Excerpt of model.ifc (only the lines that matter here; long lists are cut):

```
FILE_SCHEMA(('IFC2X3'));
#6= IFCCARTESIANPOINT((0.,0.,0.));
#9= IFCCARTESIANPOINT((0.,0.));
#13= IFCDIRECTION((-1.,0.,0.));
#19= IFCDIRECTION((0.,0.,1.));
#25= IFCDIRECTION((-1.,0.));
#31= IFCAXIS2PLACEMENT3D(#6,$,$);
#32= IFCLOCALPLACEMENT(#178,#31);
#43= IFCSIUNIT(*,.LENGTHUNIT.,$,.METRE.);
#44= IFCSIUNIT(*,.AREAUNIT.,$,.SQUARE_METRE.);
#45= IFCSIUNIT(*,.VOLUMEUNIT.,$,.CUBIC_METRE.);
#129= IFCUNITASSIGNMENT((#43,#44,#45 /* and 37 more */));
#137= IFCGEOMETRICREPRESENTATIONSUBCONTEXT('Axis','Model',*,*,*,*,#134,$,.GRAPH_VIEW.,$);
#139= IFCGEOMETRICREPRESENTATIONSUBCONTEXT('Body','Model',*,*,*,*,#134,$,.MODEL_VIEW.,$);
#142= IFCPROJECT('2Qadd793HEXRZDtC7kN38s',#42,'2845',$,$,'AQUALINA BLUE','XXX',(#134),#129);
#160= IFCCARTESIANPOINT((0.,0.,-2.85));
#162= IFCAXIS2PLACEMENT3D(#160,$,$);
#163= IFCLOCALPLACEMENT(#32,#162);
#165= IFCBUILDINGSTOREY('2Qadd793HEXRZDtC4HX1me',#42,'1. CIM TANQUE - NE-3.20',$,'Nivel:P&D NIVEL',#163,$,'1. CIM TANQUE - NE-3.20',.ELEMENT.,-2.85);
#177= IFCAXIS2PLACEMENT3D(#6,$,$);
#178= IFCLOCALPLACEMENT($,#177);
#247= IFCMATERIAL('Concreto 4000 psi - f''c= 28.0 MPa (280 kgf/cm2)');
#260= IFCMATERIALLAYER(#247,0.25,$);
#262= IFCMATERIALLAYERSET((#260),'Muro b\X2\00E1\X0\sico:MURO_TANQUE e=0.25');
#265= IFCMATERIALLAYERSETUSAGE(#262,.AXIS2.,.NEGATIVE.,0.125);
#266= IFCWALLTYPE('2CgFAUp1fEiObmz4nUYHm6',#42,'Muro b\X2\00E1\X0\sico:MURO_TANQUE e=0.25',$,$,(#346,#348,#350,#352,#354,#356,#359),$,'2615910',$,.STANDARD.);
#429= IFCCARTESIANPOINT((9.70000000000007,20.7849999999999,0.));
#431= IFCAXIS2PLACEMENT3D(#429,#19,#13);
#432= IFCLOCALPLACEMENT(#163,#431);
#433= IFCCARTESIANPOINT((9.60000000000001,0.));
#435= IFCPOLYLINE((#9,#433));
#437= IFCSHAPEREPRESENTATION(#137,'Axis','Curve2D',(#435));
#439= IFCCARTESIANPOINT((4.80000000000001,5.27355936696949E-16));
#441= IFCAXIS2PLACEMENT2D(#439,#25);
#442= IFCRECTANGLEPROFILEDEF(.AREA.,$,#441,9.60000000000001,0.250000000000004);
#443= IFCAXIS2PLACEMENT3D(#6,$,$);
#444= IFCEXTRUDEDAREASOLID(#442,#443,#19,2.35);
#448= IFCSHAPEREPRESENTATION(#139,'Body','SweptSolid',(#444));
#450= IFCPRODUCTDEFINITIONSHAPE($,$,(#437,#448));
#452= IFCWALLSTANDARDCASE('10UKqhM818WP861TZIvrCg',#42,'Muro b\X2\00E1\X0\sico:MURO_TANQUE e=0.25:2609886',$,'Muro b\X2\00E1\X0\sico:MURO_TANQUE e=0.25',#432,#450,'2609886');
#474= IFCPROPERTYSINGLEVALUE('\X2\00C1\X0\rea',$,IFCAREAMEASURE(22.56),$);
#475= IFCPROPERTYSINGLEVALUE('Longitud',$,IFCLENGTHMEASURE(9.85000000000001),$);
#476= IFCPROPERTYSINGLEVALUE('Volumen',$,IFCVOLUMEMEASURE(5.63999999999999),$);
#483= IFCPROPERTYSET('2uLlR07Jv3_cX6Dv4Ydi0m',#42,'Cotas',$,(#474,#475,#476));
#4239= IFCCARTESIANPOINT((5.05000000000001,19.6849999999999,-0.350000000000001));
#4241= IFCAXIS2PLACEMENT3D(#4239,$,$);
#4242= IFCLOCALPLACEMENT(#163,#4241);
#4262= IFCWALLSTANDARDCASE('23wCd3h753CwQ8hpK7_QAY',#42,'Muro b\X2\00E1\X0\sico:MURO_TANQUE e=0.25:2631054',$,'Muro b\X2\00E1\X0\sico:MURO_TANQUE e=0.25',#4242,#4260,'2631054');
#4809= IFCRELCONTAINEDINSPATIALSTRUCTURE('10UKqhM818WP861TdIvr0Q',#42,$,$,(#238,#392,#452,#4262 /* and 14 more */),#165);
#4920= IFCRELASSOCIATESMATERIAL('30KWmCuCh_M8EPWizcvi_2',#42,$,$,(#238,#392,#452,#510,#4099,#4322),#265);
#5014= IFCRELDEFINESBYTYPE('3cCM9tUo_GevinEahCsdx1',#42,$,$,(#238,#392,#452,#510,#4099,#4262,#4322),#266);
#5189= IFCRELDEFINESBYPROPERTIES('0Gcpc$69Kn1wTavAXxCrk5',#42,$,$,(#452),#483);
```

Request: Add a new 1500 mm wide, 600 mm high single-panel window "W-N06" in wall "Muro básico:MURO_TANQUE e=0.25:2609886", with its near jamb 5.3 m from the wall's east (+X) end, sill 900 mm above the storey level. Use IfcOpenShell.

```python
import numpy as np
import ifcopenshell
import ifcopenshell.api.feature
import ifcopenshell.api.geometry
import ifcopenshell.api.pset
import ifcopenshell.api.root
import ifcopenshell.api.spatial
import ifcopenshell.api.type
import ifcopenshell.geom
import ifcopenshell.util.element
import ifcopenshell.util.placement
import ifcopenshell.util.representation
import ifcopenshell.util.shape
import ifcopenshell.util.unit

model = ifcopenshell.open("model.ifc")
unit_scale = ifcopenshell.util.unit.calculate_unit_scale(model)
area_scale = ifcopenshell.util.unit.calculate_unit_scale(model, "AREAUNIT")
volume_scale = ifcopenshell.util.unit.calculate_unit_scale(model, "VOLUMEUNIT")
settings = ifcopenshell.geom.settings()


def volume(element):
    """Net volume in cubic metres, openings subtracted."""
    shape = ifcopenshell.geom.create_shape(settings, element)
    return ifcopenshell.util.shape.get_volume(shape.geometry)


wall = model.by_guid("10UKqhM818WP861TZIvrCg")
storey = ifcopenshell.util.element.get_container(wall, ifc_class="IfcBuildingStorey")
context = ifcopenshell.util.representation.get_context(model, "Model", "Body", "MODEL_VIEW")
before = volume(wall)

width, height, from_end, sill = 1.5, 0.6, 5.3, 0.9  # metres

# The wall runs along its own X axis, and the end named is its -X end.
wall_shape = ifcopenshell.geom.create_shape(settings, wall)
x, y, z = ifcopenshell.util.shape.get_vertices(wall_shape.geometry).T
start = x.min() + from_end
face, thickness = float(y.min()), float(y.max() - y.min())
wall_matrix = ifcopenshell.util.placement.get_local_placement(wall.ObjectPlacement)
level = ifcopenshell.util.placement.get_local_placement(storey.ObjectPlacement)[2, 3]


def in_wall(x, y):
    """Placement at x, y metres in the wall's axes, at sill height."""
    matrix = wall_matrix.copy()
    matrix[:, 3] = wall_matrix @ np.array([x / unit_scale, y / unit_scale, 0.0, 1.0])
    matrix[2, 3] = level + sill / unit_scale
    return matrix


# Opening: a box that overshoots both wall faces by 50 mm.
opening = ifcopenshell.api.root.create_entity(model, ifc_class="IfcOpeningElement")
box = ifcopenshell.api.geometry.add_wall_representation(
    model, context=context, length=width, height=height, thickness=thickness + 0.1
)
ifcopenshell.api.geometry.assign_representation(model, product=opening, representation=box)
ifcopenshell.api.geometry.edit_object_placement(model, product=opening, matrix=in_wall(start, face - 0.05), is_si=False)
ifcopenshell.api.feature.add_feature(model, feature=opening, element=wall)

window = ifcopenshell.api.root.create_entity(model, ifc_class="IfcWindow", name="W-N06")
window.OverallWidth, window.OverallHeight = width / unit_scale, height / unit_scale
body = ifcopenshell.api.geometry.add_window_representation(
    model,
    context=context,
    overall_width=window.OverallWidth,
    overall_height=window.OverallHeight,
    partition_type="SINGLE_PANEL",
)
ifcopenshell.api.geometry.assign_representation(model, product=window, representation=body)
ifcopenshell.api.spatial.assign_container(model, products=[window], relating_structure=storey)
fills = ifcopenshell.api.feature.add_filling(model, opening=opening, element=window)
fills.OwnerHistory = window.OwnerHistory  # required in IFC2X3

# IFC2X3 keeps the operation on the window style.
style = ifcopenshell.api.root.create_entity(model, ifc_class="IfcWindowStyle", name="W-N06")
style.OperationType, style.ConstructionType = "SINGLE_PANEL", "NOTDEFINED"
style.ParameterTakesPrecedence = style.Sizeable = False
ifcopenshell.api.type.assign_type(model, related_objects=[window], relating_type=style)

# Centre the window in the wall's thickness.
ifcopenshell.api.geometry.edit_object_placement(model, product=window, matrix=in_wall(start, face), is_si=False)
window_shape = ifcopenshell.geom.create_shape(settings, window)
depth = ifcopenshell.util.shape.get_vertices(window_shape.geometry)[:, 1]
offset = face + thickness / 2 - (depth.min() + depth.max()) / 2
ifcopenshell.api.geometry.edit_object_placement(model, product=window, matrix=in_wall(start, offset), is_si=False)

after = volume(wall)

# Update the wall's stored quantities.
pset = model.by_id(ifcopenshell.util.element.get_pset(wall, "Cotas", should_inherit=False)["id"])
ifcopenshell.api.pset.edit_pset(model, pset=pset, properties={
    "Área": model.create_entity("IfcAreaMeasure", after / thickness / area_scale),
    "Volumen": model.create_entity("IfcVolumeMeasure", after / volume_scale),
})

print(f"wall volume {before:.3f} -> {after:.3f} m3")

model.write("model_rev.ifc")
```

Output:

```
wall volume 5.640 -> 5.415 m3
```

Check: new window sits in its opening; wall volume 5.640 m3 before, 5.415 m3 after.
